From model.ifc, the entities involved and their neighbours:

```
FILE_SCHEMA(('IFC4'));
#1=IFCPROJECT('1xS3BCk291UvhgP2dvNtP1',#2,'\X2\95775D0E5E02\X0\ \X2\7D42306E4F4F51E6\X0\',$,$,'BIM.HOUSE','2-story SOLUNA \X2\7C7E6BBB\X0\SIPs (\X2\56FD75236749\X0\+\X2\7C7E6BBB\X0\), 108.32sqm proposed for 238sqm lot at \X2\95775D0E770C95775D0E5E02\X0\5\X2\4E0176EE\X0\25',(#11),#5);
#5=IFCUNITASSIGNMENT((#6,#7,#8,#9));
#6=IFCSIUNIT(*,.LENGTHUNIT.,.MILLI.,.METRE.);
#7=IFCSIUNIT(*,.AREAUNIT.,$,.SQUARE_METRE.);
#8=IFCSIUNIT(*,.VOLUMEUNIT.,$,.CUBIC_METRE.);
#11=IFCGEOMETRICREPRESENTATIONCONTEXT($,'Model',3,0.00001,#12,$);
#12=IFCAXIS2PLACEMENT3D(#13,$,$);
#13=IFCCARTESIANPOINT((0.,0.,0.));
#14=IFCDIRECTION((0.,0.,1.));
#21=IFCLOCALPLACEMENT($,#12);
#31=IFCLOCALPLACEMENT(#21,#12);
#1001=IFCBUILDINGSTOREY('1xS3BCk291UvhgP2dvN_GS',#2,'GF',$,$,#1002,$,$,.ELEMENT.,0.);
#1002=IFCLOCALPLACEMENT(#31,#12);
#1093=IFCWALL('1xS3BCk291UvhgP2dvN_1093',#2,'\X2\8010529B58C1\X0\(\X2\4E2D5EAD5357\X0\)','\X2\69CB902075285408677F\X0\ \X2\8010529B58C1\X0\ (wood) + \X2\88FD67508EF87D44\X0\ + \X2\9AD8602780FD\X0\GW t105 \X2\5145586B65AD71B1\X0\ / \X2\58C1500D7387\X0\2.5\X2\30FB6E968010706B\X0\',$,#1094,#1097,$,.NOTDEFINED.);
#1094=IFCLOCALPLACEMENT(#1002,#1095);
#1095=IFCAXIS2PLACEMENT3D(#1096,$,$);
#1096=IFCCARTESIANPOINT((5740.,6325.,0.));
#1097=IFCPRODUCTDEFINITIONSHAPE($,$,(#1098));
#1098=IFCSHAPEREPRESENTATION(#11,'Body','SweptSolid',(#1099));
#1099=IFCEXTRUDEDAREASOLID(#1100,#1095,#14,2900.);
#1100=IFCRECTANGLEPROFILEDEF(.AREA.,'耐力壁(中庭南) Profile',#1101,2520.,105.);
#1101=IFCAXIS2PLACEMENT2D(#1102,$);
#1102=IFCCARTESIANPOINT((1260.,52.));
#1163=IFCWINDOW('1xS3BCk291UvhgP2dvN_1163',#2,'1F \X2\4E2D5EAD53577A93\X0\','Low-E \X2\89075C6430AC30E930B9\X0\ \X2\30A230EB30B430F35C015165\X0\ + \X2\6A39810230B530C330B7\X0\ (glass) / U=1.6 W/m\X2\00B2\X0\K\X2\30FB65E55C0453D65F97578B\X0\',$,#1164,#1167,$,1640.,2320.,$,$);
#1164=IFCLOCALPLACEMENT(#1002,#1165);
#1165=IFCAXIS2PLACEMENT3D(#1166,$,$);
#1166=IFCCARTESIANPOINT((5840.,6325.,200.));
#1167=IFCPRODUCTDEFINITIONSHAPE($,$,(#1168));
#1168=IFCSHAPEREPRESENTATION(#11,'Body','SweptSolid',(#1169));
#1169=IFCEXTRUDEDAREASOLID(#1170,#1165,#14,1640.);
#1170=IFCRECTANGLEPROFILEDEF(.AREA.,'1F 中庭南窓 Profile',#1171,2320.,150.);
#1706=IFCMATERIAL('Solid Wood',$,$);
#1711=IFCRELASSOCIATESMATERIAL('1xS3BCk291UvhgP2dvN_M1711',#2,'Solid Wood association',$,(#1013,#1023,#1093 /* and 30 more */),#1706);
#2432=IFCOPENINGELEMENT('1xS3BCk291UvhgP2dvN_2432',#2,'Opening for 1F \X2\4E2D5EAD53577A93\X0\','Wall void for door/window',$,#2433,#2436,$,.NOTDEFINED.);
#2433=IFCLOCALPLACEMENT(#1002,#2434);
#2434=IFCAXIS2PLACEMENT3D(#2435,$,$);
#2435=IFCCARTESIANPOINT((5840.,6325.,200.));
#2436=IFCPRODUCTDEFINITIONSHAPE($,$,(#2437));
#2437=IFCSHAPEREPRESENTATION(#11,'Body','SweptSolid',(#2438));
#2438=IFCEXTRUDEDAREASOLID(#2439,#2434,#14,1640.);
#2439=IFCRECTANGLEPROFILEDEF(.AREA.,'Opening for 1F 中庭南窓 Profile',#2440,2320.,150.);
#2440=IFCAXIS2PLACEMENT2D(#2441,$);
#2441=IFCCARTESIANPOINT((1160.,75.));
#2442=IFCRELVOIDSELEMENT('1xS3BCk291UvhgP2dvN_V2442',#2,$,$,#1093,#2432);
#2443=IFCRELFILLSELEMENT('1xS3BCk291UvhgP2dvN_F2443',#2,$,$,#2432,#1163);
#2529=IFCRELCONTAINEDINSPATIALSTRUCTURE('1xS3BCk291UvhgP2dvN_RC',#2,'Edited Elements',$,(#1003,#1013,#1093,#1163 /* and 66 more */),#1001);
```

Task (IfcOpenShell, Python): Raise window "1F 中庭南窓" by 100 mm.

```python
import numpy as np
import ifcopenshell
import ifcopenshell.api.geometry
import ifcopenshell.util.placement
import ifcopenshell.util.unit

model = ifcopenshell.open("model.ifc")
unit_scale = ifcopenshell.util.unit.calculate_unit_scale(model)

window = model.by_guid("1xS3BCk291UvhgP2dvN_1163")
opening = window.FillsVoids[0].RelatingOpeningElement
dz = 100.0

shift = np.array([0.0, 0.0, dz])
# The window is not placed relative to its opening, so move both.
for product in (opening, window):
    matrix = ifcopenshell.util.placement.get_local_placement(product.ObjectPlacement)
    matrix[:3, 3] += shift
    ifcopenshell.api.geometry.edit_object_placement(model, product=product, matrix=matrix, is_si=False)

print(f"moved by {dz * unit_scale:+.3f} m")

model.write("model_updated.ifc")
```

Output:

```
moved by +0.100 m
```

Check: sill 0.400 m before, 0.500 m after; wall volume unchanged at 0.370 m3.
